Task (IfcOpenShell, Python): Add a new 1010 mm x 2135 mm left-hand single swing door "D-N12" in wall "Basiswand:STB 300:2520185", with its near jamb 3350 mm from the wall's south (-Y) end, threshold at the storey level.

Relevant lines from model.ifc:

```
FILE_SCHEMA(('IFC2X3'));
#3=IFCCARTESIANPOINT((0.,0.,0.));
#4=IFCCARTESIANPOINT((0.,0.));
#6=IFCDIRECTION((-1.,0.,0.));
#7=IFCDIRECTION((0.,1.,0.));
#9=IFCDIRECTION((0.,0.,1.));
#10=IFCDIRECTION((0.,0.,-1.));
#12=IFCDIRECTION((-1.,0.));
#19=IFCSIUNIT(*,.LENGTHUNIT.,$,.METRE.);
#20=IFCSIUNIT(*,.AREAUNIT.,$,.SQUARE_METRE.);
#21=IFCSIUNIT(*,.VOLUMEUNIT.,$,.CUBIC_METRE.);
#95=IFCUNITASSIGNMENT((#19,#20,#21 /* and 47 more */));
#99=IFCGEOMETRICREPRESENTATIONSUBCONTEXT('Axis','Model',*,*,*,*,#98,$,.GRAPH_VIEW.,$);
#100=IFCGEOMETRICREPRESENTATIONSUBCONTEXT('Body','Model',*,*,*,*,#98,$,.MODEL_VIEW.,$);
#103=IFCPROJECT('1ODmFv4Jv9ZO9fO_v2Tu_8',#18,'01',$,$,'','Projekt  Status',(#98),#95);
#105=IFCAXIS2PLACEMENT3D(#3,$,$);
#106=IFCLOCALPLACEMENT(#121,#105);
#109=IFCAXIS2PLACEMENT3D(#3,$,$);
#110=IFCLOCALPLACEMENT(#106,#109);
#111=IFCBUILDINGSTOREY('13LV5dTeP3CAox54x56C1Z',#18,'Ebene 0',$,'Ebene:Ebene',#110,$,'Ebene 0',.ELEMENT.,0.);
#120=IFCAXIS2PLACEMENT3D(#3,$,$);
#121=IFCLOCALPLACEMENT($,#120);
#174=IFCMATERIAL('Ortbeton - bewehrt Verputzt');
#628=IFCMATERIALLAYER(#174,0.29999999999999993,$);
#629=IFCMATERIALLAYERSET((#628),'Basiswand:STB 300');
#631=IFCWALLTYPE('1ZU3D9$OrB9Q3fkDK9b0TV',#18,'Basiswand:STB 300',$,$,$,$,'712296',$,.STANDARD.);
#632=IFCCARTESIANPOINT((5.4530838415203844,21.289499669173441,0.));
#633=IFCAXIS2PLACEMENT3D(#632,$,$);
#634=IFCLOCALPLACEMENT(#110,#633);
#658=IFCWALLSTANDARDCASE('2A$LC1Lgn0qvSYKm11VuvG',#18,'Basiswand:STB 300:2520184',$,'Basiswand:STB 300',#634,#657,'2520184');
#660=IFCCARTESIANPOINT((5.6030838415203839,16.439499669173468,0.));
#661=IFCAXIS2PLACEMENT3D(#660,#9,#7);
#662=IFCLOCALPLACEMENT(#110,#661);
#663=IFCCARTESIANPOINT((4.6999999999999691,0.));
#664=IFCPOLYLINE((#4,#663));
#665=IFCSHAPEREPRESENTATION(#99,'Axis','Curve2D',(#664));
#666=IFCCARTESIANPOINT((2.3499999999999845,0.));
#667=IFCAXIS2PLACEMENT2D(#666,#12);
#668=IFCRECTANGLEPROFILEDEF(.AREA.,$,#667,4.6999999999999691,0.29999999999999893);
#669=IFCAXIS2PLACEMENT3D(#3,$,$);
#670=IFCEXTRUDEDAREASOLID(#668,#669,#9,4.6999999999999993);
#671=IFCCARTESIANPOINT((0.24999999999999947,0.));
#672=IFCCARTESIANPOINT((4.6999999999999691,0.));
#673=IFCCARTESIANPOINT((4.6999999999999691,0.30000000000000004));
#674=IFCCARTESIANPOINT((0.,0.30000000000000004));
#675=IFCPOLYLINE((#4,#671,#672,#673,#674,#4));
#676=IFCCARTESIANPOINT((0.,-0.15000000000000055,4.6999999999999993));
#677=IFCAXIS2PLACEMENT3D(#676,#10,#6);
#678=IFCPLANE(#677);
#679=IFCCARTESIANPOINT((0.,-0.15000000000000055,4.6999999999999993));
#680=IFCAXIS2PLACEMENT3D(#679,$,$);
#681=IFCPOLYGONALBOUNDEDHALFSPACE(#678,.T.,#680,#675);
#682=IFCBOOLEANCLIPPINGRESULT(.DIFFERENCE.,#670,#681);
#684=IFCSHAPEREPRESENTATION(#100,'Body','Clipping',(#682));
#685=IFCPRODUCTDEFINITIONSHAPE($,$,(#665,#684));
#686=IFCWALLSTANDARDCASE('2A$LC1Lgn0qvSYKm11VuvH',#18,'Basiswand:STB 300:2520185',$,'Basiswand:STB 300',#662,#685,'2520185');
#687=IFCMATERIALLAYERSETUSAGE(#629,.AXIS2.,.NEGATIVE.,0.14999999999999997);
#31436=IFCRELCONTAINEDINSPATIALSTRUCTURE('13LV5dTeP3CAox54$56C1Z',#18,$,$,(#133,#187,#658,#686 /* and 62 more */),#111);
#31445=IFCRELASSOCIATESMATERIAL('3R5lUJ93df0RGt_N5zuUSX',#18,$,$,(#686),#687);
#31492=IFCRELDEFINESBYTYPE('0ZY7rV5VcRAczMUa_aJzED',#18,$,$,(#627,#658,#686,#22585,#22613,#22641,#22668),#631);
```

```python
import numpy as np
import ifcopenshell
import ifcopenshell.api.feature
import ifcopenshell.api.geometry
import ifcopenshell.api.root
import ifcopenshell.api.spatial
import ifcopenshell.api.type
import ifcopenshell.geom
import ifcopenshell.util.element
import ifcopenshell.util.placement
import ifcopenshell.util.representation
import ifcopenshell.util.shape
import ifcopenshell.util.unit

model = ifcopenshell.open("model.ifc")
unit_scale = ifcopenshell.util.unit.calculate_unit_scale(model)
settings = ifcopenshell.geom.settings()


def volume(element):
    """Net volume in cubic metres, openings subtracted."""
    shape = ifcopenshell.geom.create_shape(settings, element)
    return ifcopenshell.util.shape.get_volume(shape.geometry)


wall = model.by_guid("2A$LC1Lgn0qvSYKm11VuvH")
storey = ifcopenshell.util.element.get_container(wall, ifc_class="IfcBuildingStorey")
context = ifcopenshell.util.representation.get_context(model, "Model", "Body", "MODEL_VIEW")
before = volume(wall)

width, height, from_end, sill = 1.01, 2.135, 3.35, 0.0  # metres

# The wall runs along its own X axis, and the end named is its -X end.
wall_shape = ifcopenshell.geom.create_shape(settings, wall)
x, y, z = ifcopenshell.util.shape.get_vertices(wall_shape.geometry).T
start = x.min() + from_end
face, thickness = float(y.min()), float(y.max() - y.min())
wall_matrix = ifcopenshell.util.placement.get_local_placement(wall.ObjectPlacement)
level = ifcopenshell.util.placement.get_local_placement(storey.ObjectPlacement)[2, 3]


def in_wall(x, y):
    """Placement at x, y metres in the wall's axes, at sill height."""
    matrix = wall_matrix.copy()
    matrix[:, 3] = wall_matrix @ np.array([x / unit_scale, y / unit_scale, 0.0, 1.0])
    matrix[2, 3] = level + sill / unit_scale
    return matrix


# Opening: a box that overshoots both wall faces by 50 mm.
opening = ifcopenshell.api.root.create_entity(model, ifc_class="IfcOpeningElement")
box = ifcopenshell.api.geometry.add_wall_representation(
    model, context=context, length=width, height=height, thickness=thickness + 0.1
)
ifcopenshell.api.geometry.assign_representation(model, product=opening, representation=box)
ifcopenshell.api.geometry.edit_object_placement(model, product=opening, matrix=in_wall(start, face - 0.05), is_si=False)
ifcopenshell.api.feature.add_feature(model, feature=opening, element=wall)

door = ifcopenshell.api.root.create_entity(model, ifc_class="IfcDoor", name="D-N12")
door.OverallWidth, door.OverallHeight = width / unit_scale, height / unit_scale
body = ifcopenshell.api.geometry.add_door_representation(
    model,
    context=context,
    overall_width=door.OverallWidth,
    overall_height=door.OverallHeight,
    operation_type="SINGLE_SWING_LEFT",
    lining_properties={"LiningDepth": thickness / unit_scale, "ThresholdDepth": thickness / unit_scale},
)
ifcopenshell.api.geometry.assign_representation(model, product=door, representation=body)
ifcopenshell.api.spatial.assign_container(model, products=[door], relating_structure=storey)
fills = ifcopenshell.api.feature.add_filling(model, opening=opening, element=door)
fills.OwnerHistory = door.OwnerHistory  # required in IFC2X3

# IFC2X3 keeps the operation on the door style.
style = ifcopenshell.api.root.create_entity(model, ifc_class="IfcDoorStyle", name="D-N12")
style.OperationType, style.ConstructionType = "SINGLE_SWING_LEFT", "NOTDEFINED"
style.ParameterTakesPrecedence = style.Sizeable = False
ifcopenshell.api.type.assign_type(model, related_objects=[door], relating_type=style)

# The lining spans the wall, so the door starts at the wall face.
ifcopenshell.api.geometry.edit_object_placement(model, product=door, matrix=in_wall(start, face), is_si=False)

after = volume(wall)

print(f"wall volume {before:.3f} -> {after:.3f} m3")

model.write("model_rev.ifc")
```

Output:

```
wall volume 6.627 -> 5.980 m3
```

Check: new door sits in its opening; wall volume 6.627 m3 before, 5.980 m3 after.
